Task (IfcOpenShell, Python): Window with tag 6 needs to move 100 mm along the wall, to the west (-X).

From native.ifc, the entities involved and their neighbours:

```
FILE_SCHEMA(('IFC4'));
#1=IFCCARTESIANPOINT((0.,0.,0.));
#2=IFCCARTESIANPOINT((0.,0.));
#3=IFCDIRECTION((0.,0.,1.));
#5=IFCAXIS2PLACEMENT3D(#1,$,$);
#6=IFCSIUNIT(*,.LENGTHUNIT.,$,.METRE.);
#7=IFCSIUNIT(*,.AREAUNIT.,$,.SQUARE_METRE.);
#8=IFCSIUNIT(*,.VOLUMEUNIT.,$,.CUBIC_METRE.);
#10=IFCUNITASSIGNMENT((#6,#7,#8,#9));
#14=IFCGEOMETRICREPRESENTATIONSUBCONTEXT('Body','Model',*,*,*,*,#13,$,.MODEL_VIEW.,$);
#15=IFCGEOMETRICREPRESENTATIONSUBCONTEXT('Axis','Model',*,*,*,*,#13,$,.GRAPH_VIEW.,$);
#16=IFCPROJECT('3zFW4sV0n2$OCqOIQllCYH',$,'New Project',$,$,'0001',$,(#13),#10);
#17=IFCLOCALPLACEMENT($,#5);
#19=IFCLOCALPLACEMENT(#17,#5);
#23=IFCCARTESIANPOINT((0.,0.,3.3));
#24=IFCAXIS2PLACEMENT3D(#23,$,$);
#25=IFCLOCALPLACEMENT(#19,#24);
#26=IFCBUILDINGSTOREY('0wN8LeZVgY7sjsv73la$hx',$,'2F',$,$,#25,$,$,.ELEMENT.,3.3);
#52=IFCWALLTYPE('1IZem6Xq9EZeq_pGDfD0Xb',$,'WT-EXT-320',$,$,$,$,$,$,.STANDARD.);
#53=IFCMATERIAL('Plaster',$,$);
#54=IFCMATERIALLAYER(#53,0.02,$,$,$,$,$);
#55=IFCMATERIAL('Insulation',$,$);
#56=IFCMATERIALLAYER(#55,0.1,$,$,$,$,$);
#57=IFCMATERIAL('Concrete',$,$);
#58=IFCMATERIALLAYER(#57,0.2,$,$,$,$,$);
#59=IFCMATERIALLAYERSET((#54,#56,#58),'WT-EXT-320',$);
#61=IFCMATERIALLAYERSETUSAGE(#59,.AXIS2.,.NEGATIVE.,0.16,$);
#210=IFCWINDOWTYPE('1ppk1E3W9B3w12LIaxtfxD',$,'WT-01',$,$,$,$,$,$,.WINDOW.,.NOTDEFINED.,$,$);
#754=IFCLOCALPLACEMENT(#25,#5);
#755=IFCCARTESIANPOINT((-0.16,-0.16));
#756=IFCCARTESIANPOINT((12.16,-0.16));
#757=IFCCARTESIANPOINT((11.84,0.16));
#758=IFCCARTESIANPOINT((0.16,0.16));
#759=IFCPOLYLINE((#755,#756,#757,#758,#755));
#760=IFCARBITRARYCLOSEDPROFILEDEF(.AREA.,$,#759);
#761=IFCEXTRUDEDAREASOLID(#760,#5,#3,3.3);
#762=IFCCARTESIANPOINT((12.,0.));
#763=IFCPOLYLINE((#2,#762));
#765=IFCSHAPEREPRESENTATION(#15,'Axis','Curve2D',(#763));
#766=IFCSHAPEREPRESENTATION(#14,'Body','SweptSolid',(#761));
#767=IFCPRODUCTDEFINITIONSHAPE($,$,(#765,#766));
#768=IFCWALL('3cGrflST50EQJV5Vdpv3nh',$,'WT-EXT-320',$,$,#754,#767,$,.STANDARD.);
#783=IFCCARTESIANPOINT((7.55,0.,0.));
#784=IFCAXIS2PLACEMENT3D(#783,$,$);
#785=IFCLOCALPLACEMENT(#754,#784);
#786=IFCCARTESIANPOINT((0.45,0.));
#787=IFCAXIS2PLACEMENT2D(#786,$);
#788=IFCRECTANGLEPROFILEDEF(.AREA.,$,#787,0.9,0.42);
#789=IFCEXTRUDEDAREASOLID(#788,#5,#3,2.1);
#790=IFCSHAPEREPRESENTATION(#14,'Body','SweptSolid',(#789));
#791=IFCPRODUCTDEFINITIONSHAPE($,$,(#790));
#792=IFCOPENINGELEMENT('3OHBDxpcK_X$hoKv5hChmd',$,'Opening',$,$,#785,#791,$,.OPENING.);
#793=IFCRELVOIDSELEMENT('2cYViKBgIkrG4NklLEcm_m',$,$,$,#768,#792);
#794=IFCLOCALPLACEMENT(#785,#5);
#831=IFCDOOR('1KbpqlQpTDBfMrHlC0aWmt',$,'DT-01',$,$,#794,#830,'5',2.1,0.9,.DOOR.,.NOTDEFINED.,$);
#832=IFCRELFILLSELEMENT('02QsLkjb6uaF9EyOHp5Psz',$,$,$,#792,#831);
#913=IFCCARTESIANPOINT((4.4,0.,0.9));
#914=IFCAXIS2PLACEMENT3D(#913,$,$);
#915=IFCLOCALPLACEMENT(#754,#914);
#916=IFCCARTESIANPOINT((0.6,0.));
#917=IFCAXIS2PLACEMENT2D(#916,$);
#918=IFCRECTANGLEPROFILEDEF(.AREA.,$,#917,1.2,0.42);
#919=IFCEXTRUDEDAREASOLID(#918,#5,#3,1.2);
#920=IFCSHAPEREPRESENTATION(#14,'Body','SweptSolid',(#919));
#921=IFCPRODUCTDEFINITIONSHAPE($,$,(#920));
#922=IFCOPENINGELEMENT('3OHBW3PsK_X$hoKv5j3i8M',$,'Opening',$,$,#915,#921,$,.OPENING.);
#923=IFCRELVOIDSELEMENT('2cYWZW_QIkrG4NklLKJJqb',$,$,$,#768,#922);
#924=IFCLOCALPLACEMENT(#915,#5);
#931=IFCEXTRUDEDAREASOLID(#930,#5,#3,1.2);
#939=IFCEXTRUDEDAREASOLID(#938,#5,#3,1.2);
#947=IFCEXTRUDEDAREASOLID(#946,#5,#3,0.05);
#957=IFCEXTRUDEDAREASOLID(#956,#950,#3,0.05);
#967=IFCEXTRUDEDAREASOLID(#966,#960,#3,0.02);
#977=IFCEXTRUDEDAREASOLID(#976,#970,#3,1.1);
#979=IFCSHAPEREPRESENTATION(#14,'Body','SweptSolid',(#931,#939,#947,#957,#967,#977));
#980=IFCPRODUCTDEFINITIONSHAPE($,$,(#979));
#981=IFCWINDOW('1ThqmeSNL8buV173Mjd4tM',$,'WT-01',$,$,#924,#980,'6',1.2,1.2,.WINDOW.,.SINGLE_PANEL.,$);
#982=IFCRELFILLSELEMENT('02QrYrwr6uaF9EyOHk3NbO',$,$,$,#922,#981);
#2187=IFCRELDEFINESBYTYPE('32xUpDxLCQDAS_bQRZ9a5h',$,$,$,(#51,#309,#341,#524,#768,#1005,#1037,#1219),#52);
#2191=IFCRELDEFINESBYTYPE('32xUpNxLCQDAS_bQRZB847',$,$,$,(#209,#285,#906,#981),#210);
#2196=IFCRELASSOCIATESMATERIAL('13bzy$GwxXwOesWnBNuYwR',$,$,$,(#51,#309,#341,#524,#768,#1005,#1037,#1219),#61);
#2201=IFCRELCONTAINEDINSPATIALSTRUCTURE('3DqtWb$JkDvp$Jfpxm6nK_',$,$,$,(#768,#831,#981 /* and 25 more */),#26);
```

```python
import ifcopenshell
import ifcopenshell.api.geometry
import ifcopenshell.util.placement
import ifcopenshell.util.unit

model = ifcopenshell.open("native.ifc")
unit_scale = ifcopenshell.util.unit.calculate_unit_scale(model)

window = model.by_guid("1ThqmeSNL8buV173Mjd4tM")
opening = window.FillsVoids[0].RelatingOpeningElement
wall = opening.VoidsElements[0].RelatingBuildingElement

wall_matrix = ifcopenshell.util.placement.get_local_placement(wall.ObjectPlacement)
shift = wall_matrix[:3, 0] * -0.1 / unit_scale
before = ifcopenshell.util.placement.get_local_placement(window.ObjectPlacement)[:3, 3].copy()

# The window is placed relative to its opening, so it follows when the opening moves.
matrix = ifcopenshell.util.placement.get_local_placement(opening.ObjectPlacement)
matrix[:3, 3] += shift
ifcopenshell.api.geometry.edit_object_placement(
    model, product=opening, matrix=matrix, is_si=False, should_transform_children=True
)

after = ifcopenshell.util.placement.get_local_placement(window.ObjectPlacement)[:3, 3]
print("window moved by", (after - before).round(3) + 0.0)

model.write("native_edited.ifc")
```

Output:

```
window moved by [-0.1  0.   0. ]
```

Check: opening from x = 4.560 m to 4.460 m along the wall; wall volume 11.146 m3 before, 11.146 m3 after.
